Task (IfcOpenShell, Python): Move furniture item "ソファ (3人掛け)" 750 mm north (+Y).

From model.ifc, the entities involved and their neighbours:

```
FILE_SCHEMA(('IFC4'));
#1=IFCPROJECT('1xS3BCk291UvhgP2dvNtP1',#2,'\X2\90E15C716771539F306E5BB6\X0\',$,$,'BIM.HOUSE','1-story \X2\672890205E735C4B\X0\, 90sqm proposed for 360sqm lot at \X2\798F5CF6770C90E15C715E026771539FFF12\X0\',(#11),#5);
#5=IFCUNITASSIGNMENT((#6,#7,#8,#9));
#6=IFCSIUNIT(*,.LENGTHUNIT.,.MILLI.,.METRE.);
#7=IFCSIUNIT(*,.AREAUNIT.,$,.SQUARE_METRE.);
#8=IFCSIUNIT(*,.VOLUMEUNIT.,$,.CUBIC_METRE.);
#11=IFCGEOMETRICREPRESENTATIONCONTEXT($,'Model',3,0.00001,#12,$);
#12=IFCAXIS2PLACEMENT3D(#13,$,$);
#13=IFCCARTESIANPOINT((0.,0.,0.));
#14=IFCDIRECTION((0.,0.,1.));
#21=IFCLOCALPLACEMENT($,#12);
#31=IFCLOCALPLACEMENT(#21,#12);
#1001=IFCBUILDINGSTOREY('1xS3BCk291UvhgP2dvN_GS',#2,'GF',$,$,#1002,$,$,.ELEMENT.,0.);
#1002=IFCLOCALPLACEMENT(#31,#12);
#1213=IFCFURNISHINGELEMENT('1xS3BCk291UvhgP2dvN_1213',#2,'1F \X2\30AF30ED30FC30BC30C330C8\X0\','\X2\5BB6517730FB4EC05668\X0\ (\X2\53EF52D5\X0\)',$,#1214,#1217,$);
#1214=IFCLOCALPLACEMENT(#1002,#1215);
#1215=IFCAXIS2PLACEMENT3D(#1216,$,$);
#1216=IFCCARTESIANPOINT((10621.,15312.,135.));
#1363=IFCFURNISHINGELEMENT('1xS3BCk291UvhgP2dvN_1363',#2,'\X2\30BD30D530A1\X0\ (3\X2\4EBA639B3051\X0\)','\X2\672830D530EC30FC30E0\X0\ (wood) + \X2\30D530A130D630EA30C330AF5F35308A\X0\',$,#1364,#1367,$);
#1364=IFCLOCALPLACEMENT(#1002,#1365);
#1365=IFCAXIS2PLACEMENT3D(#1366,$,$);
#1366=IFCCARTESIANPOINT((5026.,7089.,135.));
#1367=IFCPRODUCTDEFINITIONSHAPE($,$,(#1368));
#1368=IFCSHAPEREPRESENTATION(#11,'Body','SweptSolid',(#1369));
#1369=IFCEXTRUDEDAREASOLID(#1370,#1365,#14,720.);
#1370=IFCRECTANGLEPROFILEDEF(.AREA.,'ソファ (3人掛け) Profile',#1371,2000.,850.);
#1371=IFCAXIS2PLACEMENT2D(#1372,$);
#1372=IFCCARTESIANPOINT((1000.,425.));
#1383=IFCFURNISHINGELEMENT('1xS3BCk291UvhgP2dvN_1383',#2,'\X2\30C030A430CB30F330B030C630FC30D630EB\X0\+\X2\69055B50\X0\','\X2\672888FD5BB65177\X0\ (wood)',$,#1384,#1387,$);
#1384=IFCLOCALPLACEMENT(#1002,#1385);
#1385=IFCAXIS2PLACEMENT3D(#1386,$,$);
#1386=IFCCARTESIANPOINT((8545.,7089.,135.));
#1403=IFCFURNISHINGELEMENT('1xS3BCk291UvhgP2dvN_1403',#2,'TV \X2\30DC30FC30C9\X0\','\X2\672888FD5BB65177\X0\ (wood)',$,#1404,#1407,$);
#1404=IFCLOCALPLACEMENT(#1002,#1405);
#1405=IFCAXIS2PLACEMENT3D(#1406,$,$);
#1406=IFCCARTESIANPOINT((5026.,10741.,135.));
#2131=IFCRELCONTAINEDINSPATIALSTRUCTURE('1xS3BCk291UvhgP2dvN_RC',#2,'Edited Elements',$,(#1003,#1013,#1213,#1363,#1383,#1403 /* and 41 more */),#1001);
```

```python
import ifcopenshell
import ifcopenshell.api.geometry
import ifcopenshell.util.placement
import ifcopenshell.util.unit

model = ifcopenshell.open("model.ifc")
unit_scale = ifcopenshell.util.unit.calculate_unit_scale(model)

item = model.by_id(1363)
matrix = ifcopenshell.util.placement.get_local_placement(item.ObjectPlacement)
matrix[1, 3] += 0.75 / unit_scale
ifcopenshell.api.geometry.edit_object_placement(model, product=item, matrix=matrix, is_si=False)

print(ifcopenshell.util.placement.get_local_placement(item.ObjectPlacement).round(3) + 0.0)

model.write("model_updated.ifc")
```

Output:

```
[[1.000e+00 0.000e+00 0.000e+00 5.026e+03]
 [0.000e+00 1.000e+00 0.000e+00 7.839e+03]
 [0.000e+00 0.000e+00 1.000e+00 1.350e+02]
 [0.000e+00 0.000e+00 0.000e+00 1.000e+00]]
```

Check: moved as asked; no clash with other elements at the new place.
